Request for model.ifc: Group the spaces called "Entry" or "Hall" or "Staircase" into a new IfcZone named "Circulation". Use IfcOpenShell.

First a look at what the model holds.

```python
import ifcopenshell

model = ifcopenshell.open("model.ifc")
print(model.schema)
seen = {}
for space in model.by_type("IfcSpace"):
    seen[space.LongName] = seen.get(space.LongName, 0) + 1
for name, count in sorted(seen.items(), key=str):
    print(count, "x", name)
print("zones:", [z.Name for z in model.by_type("IfcZone")][:20])
```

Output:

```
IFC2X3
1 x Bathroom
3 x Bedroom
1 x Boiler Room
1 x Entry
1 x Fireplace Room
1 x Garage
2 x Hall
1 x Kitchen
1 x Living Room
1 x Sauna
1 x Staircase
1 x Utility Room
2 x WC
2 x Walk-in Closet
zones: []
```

```python
import ifcopenshell
import ifcopenshell.api.group
import ifcopenshell.api.root

model = ifcopenshell.open("model.ifc")

names = {"Entry", "Hall", "Staircase"}
spaces = [s for s in model.by_type("IfcSpace") if s.LongName in names]

zone = ifcopenshell.api.root.create_entity(model, ifc_class="IfcZone", name="Circulation")
ifcopenshell.api.group.assign_group(model, products=spaces, group=zone)
print(len(spaces), "spaces in", zone.Name)

model.write("model_updated.ifc")
```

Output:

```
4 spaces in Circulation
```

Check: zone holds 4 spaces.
